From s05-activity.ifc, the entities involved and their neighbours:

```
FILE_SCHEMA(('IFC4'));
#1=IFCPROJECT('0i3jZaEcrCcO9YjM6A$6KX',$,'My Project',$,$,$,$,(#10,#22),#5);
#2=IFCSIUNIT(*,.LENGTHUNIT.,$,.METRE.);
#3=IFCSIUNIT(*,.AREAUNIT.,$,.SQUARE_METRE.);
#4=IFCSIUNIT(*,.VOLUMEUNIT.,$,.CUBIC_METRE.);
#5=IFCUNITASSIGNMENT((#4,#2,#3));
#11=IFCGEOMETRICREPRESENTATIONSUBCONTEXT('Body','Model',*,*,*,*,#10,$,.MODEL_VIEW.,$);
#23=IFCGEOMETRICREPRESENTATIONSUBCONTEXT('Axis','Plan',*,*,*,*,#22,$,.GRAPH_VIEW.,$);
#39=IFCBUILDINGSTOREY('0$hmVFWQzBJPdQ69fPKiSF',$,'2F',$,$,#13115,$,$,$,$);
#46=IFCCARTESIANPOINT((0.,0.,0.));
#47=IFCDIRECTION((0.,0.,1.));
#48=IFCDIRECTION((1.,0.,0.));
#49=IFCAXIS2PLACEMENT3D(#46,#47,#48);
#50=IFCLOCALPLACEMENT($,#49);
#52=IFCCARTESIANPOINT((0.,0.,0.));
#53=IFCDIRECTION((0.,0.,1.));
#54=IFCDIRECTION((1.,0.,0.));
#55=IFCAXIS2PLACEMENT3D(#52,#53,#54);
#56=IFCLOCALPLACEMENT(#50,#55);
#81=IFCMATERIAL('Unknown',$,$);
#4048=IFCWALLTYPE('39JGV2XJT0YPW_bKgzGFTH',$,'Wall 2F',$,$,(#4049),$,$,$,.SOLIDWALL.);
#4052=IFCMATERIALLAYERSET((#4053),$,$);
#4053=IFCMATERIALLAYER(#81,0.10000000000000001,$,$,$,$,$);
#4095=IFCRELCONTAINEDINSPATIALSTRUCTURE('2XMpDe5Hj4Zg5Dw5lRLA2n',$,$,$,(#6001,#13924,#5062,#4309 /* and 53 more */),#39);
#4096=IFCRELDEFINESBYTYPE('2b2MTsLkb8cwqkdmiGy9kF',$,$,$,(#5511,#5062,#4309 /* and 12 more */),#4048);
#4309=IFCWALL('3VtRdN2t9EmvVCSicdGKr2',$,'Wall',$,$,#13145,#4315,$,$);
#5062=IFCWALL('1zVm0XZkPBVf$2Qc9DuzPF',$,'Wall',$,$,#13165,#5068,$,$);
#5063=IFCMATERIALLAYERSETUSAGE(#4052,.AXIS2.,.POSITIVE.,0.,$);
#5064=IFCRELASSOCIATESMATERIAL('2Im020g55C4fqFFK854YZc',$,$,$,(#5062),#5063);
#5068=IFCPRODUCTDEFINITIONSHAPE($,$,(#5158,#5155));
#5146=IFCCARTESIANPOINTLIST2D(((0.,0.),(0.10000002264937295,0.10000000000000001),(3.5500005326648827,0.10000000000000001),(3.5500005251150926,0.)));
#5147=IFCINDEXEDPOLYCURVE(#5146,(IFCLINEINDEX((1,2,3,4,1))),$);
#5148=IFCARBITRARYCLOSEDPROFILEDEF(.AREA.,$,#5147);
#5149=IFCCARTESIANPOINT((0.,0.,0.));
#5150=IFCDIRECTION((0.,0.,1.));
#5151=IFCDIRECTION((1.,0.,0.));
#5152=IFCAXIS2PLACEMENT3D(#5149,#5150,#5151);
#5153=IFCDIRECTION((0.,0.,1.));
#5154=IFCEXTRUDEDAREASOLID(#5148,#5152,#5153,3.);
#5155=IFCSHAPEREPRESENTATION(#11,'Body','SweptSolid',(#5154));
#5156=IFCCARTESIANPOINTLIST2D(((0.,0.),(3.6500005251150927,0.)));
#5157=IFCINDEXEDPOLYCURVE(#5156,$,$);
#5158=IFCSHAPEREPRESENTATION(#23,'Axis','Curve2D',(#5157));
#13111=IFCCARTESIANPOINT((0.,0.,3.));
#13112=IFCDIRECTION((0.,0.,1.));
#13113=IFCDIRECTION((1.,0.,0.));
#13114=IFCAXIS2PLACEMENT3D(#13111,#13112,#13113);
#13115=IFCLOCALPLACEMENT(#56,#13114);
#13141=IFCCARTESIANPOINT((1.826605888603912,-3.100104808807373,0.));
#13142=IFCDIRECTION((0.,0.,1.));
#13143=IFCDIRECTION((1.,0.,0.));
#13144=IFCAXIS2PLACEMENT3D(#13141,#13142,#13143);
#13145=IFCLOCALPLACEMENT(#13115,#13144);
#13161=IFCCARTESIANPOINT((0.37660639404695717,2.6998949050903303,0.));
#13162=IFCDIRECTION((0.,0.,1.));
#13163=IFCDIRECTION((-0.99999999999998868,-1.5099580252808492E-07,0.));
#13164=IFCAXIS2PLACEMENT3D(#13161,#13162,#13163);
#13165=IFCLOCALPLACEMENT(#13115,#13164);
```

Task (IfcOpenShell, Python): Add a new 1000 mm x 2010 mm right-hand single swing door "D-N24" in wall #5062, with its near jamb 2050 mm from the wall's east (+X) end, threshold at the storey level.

```python
import numpy as np
import ifcopenshell
import ifcopenshell.api.feature
import ifcopenshell.api.geometry
import ifcopenshell.api.root
import ifcopenshell.api.spatial
import ifcopenshell.geom
import ifcopenshell.util.element
import ifcopenshell.util.placement
import ifcopenshell.util.representation
import ifcopenshell.util.shape
import ifcopenshell.util.unit

model = ifcopenshell.open("s05-activity.ifc")
unit_scale = ifcopenshell.util.unit.calculate_unit_scale(model)
settings = ifcopenshell.geom.settings()


def volume(element):
    """Net volume in cubic metres, openings subtracted."""
    shape = ifcopenshell.geom.create_shape(settings, element)
    return ifcopenshell.util.shape.get_volume(shape.geometry)


wall = model.by_id(5062)
storey = ifcopenshell.util.element.get_container(wall, ifc_class="IfcBuildingStorey")
context = ifcopenshell.util.representation.get_context(model, "Model", "Body", "MODEL_VIEW")
before = volume(wall)

width, height, from_end, sill = 1, 2.01, 2.05, 0.0  # metres

# The wall runs along its own X axis, and the end named is its -X end.
wall_shape = ifcopenshell.geom.create_shape(settings, wall)
x, y, z = ifcopenshell.util.shape.get_vertices(wall_shape.geometry).T
start = x.min() + from_end
face, thickness = float(y.min()), float(y.max() - y.min())
wall_matrix = ifcopenshell.util.placement.get_local_placement(wall.ObjectPlacement)
level = ifcopenshell.util.placement.get_local_placement(storey.ObjectPlacement)[2, 3]


def in_wall(x, y):
    """Placement at x, y metres in the wall's axes, at sill height."""
    matrix = wall_matrix.copy()
    matrix[:, 3] = wall_matrix @ np.array([x / unit_scale, y / unit_scale, 0.0, 1.0])
    matrix[2, 3] = level + sill / unit_scale
    return matrix


# Opening: a box that overshoots both wall faces by 50 mm.
opening = ifcopenshell.api.root.create_entity(model, ifc_class="IfcOpeningElement", predefined_type="OPENING")
box = ifcopenshell.api.geometry.add_wall_representation(
    model, context=context, length=width, height=height, thickness=thickness + 0.1
)
ifcopenshell.api.geometry.assign_representation(model, product=opening, representation=box)
ifcopenshell.api.geometry.edit_object_placement(model, product=opening, matrix=in_wall(start, face - 0.05), is_si=False)
ifcopenshell.api.feature.add_feature(model, feature=opening, element=wall)

door = ifcopenshell.api.root.create_entity(model, ifc_class="IfcDoor", name="D-N24", predefined_type="DOOR")
door.OverallWidth, door.OverallHeight = width / unit_scale, height / unit_scale
door.OperationType = "SINGLE_SWING_RIGHT"
body = ifcopenshell.api.geometry.add_door_representation(
    model,
    context=context,
    overall_width=door.OverallWidth,
    overall_height=door.OverallHeight,
    operation_type="SINGLE_SWING_RIGHT",
    lining_properties={"LiningDepth": thickness / unit_scale, "ThresholdDepth": thickness / unit_scale},
)
ifcopenshell.api.geometry.assign_representation(model, product=door, representation=body)
ifcopenshell.api.spatial.assign_container(model, products=[door], relating_structure=storey)
ifcopenshell.api.feature.add_filling(model, opening=opening, element=door)

# The lining spans the wall, so the door starts at the wall face.
ifcopenshell.api.geometry.edit_object_placement(model, product=door, matrix=in_wall(start, face), is_si=False)

after = volume(wall)

print(f"wall volume {before:.3f} -> {after:.3f} m3")

model.write("s05-activity-out.ifc")
```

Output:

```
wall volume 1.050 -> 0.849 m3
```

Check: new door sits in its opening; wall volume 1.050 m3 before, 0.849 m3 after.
